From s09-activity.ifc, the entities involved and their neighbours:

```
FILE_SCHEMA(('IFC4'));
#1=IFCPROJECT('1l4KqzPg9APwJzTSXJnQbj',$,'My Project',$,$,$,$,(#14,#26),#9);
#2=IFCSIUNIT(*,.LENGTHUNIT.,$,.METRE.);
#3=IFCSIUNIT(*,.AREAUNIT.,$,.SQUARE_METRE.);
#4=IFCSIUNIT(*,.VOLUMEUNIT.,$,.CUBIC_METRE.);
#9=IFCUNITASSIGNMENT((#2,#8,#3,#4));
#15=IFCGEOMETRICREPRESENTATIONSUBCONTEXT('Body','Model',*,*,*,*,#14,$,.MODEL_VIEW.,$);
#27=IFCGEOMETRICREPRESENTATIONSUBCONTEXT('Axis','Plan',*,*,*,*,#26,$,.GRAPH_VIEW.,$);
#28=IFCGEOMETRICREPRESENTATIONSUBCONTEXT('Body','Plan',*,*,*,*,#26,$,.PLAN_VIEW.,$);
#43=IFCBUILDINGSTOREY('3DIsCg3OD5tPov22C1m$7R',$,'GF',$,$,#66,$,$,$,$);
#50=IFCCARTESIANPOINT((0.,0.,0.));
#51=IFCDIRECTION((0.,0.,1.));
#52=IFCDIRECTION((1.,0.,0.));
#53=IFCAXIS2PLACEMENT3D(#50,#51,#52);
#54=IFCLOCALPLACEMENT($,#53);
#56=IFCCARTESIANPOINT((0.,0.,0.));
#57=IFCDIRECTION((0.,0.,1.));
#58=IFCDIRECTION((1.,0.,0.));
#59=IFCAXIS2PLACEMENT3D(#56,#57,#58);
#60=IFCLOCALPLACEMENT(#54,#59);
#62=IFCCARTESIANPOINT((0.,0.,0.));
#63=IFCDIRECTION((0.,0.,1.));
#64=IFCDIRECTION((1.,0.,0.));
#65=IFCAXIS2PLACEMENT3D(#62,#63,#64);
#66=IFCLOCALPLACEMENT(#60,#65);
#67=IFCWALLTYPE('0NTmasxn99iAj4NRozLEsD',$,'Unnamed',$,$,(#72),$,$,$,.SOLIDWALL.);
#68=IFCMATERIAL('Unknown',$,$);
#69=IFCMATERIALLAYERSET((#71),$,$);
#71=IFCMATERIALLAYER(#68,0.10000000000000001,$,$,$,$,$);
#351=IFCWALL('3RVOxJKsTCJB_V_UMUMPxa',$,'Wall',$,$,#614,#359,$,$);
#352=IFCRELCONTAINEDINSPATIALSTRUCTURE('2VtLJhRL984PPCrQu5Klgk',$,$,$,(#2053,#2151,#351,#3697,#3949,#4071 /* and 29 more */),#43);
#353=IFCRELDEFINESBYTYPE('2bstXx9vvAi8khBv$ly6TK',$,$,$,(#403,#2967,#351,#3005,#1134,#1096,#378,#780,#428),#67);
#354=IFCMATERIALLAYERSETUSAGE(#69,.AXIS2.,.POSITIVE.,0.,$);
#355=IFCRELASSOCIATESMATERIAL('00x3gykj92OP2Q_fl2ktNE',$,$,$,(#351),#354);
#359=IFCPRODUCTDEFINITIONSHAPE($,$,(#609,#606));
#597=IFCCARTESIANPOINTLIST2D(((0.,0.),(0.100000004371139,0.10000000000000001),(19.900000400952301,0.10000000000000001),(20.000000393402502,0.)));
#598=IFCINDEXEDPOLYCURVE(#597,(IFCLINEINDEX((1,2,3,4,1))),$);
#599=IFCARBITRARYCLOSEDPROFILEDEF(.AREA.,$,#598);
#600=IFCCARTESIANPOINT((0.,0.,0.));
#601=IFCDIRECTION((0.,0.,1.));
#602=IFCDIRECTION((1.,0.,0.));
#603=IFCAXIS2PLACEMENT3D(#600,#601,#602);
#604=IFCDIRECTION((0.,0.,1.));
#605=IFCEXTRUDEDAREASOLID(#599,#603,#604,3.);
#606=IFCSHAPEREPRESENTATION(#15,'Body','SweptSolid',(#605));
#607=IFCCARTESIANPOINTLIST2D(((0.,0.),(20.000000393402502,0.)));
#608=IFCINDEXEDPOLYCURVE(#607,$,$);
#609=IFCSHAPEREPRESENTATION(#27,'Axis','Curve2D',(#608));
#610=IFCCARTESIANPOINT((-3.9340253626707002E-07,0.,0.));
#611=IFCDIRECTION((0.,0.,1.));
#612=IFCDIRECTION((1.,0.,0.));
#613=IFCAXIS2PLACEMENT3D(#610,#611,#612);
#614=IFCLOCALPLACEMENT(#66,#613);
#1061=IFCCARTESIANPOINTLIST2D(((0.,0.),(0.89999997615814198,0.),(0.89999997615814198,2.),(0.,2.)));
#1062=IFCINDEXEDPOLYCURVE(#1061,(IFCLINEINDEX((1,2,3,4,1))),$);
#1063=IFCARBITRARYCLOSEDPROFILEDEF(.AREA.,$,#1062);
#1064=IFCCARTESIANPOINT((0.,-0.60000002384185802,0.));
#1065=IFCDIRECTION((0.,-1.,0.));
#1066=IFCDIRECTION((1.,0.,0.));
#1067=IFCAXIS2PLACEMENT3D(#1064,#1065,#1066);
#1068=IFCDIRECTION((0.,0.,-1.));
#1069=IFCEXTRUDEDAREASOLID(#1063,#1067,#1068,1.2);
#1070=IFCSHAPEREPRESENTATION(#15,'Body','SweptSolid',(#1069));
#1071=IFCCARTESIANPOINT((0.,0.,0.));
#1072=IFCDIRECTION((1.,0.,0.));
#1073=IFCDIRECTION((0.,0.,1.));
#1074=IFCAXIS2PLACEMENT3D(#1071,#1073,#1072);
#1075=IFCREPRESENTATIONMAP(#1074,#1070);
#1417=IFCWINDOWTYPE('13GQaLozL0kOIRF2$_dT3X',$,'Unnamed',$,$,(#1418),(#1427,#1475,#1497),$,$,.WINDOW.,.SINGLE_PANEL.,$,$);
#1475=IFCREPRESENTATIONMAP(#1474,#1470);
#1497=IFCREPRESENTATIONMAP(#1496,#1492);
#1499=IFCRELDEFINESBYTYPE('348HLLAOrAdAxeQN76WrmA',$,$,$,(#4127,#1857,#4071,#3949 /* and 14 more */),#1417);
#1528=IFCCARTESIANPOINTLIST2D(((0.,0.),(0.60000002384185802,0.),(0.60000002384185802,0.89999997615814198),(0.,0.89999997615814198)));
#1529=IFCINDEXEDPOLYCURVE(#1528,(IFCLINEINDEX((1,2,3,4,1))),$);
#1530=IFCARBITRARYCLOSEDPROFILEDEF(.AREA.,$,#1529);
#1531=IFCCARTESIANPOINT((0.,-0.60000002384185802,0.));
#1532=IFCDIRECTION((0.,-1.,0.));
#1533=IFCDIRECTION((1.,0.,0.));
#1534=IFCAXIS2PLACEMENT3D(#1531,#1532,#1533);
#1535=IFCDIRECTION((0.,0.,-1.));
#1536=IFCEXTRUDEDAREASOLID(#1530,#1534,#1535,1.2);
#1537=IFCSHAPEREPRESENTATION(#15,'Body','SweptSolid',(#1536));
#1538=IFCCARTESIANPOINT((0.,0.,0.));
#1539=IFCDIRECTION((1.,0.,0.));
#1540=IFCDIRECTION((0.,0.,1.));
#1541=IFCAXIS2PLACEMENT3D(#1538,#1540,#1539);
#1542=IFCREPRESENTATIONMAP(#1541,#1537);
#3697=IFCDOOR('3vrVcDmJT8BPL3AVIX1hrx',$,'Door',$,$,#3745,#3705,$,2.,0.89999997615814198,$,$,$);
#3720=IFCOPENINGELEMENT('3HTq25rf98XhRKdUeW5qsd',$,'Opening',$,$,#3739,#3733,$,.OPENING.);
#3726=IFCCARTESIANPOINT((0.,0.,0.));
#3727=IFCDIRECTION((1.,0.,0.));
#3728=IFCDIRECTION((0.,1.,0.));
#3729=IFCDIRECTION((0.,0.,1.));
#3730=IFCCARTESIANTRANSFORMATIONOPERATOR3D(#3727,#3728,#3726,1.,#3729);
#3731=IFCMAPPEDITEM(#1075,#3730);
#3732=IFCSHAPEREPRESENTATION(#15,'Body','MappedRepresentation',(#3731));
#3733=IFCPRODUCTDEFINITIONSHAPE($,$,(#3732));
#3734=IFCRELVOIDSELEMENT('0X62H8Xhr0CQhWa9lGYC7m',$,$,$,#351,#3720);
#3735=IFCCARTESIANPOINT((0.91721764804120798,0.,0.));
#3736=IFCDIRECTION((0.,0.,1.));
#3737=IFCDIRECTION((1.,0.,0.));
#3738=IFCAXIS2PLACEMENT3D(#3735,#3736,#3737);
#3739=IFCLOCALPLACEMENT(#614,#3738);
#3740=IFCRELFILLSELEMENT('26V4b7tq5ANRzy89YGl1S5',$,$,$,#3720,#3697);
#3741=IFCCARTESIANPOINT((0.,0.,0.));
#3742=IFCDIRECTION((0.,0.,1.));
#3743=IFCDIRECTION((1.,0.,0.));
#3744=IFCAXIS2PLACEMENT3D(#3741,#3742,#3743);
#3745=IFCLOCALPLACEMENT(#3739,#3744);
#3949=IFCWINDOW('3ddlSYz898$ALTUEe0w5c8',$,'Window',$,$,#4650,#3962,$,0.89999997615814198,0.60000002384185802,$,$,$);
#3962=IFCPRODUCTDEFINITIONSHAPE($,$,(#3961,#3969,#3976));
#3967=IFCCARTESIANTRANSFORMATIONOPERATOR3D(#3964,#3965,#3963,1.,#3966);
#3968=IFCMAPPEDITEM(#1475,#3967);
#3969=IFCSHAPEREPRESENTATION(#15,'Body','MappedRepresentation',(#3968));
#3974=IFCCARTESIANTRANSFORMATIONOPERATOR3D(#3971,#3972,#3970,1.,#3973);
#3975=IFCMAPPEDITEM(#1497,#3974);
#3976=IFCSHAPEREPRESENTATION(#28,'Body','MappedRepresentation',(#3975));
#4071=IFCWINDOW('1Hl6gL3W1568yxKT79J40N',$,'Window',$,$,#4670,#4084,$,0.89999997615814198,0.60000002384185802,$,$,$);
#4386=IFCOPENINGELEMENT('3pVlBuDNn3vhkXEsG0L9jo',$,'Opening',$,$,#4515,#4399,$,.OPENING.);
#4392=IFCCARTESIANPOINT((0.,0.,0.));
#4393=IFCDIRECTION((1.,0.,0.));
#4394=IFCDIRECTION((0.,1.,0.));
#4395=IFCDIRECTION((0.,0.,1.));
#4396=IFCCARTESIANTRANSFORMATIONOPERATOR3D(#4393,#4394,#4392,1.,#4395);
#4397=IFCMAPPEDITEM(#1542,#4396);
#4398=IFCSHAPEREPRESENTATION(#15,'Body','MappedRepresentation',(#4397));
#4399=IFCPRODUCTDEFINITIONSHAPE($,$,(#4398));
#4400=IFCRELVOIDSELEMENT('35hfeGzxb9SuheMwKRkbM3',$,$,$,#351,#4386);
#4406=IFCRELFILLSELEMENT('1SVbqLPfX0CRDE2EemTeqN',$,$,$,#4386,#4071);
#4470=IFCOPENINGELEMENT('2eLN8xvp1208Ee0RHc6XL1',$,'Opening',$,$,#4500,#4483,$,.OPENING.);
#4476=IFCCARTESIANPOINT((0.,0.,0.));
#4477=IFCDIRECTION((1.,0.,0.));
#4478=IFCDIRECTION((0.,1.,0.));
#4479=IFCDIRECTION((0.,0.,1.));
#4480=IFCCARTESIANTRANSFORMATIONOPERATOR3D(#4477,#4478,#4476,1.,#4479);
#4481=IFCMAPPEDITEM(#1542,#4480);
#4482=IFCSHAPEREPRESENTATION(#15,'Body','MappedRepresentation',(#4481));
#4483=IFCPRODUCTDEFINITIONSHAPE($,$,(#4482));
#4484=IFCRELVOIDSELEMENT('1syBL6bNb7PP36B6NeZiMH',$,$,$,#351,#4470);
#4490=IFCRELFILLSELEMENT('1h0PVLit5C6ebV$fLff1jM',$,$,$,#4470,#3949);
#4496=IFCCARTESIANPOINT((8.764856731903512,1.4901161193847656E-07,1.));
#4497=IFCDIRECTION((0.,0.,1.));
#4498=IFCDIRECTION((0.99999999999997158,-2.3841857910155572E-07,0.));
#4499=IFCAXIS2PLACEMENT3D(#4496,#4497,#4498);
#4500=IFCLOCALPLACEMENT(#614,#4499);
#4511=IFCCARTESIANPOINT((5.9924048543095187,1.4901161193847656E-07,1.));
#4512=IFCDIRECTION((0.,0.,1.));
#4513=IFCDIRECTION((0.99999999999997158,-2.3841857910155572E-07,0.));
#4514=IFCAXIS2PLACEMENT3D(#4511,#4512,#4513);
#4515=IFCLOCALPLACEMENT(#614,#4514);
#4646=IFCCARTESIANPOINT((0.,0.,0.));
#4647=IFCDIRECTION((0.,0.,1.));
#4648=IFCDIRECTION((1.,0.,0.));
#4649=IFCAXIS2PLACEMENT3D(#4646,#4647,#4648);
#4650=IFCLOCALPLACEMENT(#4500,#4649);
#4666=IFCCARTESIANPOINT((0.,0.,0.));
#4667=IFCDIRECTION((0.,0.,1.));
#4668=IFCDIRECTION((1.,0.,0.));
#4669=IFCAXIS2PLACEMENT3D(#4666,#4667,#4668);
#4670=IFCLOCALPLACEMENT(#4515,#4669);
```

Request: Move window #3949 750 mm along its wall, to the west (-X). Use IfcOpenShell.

```python
import ifcopenshell
import ifcopenshell.api.geometry
import ifcopenshell.util.placement
import ifcopenshell.util.unit

model = ifcopenshell.open("s09-activity.ifc")
unit_scale = ifcopenshell.util.unit.calculate_unit_scale(model)

window = model.by_id(3949)
opening = window.FillsVoids[0].RelatingOpeningElement
wall = opening.VoidsElements[0].RelatingBuildingElement

wall_matrix = ifcopenshell.util.placement.get_local_placement(wall.ObjectPlacement)
shift = wall_matrix[:3, 0] * -0.75 / unit_scale
before = ifcopenshell.util.placement.get_local_placement(window.ObjectPlacement)[:3, 3].copy()

# The window is placed relative to its opening, so it follows when the opening moves.
matrix = ifcopenshell.util.placement.get_local_placement(opening.ObjectPlacement)
matrix[:3, 3] += shift
ifcopenshell.api.geometry.edit_object_placement(
    model, product=opening, matrix=matrix, is_si=False, should_transform_children=True
)

after = ifcopenshell.util.placement.get_local_placement(window.ObjectPlacement)[:3, 3]
print("window moved by", (after - before).round(3) + 0.0)

model.write("s09-activity_updated.ifc")
```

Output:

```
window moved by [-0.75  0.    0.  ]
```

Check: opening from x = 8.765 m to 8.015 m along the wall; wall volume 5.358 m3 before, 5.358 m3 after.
